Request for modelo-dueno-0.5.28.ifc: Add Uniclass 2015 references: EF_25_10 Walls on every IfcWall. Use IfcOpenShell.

First a look at what the model holds.

```python
import ifcopenshell

model = ifcopenshell.open("modelo-dueno-0.5.28.ifc")
print(model.schema)
print("classifications:", [c.Name for c in model.by_type("IfcClassification")])
for ifc_class in ("IfcDoor", "IfcRoof", "IfcStair", "IfcWall", "IfcWindow"):
    print(ifc_class, len(model.by_type(ifc_class)))
```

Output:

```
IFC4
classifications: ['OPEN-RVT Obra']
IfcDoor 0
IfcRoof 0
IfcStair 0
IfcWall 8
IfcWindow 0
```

```python
import ifcopenshell
import ifcopenshell.api.classification

model = ifcopenshell.open("modelo-dueno-0.5.28.ifc")

system = ifcopenshell.api.classification.add_classification(model, classification="Uniclass 2015")

codes = {
    "IfcWall": ("EF_25_10", "Walls"),
}
for ifc_class, (code, name) in codes.items():
    products = model.by_type(ifc_class)
    ifcopenshell.api.classification.add_reference(
        model, products=products, classification=system, identification=code, name=name
    )
    print(code, len(products))

model.write("modelo-dueno-0.5.28-out.ifc")
```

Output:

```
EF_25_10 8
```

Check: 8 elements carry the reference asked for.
